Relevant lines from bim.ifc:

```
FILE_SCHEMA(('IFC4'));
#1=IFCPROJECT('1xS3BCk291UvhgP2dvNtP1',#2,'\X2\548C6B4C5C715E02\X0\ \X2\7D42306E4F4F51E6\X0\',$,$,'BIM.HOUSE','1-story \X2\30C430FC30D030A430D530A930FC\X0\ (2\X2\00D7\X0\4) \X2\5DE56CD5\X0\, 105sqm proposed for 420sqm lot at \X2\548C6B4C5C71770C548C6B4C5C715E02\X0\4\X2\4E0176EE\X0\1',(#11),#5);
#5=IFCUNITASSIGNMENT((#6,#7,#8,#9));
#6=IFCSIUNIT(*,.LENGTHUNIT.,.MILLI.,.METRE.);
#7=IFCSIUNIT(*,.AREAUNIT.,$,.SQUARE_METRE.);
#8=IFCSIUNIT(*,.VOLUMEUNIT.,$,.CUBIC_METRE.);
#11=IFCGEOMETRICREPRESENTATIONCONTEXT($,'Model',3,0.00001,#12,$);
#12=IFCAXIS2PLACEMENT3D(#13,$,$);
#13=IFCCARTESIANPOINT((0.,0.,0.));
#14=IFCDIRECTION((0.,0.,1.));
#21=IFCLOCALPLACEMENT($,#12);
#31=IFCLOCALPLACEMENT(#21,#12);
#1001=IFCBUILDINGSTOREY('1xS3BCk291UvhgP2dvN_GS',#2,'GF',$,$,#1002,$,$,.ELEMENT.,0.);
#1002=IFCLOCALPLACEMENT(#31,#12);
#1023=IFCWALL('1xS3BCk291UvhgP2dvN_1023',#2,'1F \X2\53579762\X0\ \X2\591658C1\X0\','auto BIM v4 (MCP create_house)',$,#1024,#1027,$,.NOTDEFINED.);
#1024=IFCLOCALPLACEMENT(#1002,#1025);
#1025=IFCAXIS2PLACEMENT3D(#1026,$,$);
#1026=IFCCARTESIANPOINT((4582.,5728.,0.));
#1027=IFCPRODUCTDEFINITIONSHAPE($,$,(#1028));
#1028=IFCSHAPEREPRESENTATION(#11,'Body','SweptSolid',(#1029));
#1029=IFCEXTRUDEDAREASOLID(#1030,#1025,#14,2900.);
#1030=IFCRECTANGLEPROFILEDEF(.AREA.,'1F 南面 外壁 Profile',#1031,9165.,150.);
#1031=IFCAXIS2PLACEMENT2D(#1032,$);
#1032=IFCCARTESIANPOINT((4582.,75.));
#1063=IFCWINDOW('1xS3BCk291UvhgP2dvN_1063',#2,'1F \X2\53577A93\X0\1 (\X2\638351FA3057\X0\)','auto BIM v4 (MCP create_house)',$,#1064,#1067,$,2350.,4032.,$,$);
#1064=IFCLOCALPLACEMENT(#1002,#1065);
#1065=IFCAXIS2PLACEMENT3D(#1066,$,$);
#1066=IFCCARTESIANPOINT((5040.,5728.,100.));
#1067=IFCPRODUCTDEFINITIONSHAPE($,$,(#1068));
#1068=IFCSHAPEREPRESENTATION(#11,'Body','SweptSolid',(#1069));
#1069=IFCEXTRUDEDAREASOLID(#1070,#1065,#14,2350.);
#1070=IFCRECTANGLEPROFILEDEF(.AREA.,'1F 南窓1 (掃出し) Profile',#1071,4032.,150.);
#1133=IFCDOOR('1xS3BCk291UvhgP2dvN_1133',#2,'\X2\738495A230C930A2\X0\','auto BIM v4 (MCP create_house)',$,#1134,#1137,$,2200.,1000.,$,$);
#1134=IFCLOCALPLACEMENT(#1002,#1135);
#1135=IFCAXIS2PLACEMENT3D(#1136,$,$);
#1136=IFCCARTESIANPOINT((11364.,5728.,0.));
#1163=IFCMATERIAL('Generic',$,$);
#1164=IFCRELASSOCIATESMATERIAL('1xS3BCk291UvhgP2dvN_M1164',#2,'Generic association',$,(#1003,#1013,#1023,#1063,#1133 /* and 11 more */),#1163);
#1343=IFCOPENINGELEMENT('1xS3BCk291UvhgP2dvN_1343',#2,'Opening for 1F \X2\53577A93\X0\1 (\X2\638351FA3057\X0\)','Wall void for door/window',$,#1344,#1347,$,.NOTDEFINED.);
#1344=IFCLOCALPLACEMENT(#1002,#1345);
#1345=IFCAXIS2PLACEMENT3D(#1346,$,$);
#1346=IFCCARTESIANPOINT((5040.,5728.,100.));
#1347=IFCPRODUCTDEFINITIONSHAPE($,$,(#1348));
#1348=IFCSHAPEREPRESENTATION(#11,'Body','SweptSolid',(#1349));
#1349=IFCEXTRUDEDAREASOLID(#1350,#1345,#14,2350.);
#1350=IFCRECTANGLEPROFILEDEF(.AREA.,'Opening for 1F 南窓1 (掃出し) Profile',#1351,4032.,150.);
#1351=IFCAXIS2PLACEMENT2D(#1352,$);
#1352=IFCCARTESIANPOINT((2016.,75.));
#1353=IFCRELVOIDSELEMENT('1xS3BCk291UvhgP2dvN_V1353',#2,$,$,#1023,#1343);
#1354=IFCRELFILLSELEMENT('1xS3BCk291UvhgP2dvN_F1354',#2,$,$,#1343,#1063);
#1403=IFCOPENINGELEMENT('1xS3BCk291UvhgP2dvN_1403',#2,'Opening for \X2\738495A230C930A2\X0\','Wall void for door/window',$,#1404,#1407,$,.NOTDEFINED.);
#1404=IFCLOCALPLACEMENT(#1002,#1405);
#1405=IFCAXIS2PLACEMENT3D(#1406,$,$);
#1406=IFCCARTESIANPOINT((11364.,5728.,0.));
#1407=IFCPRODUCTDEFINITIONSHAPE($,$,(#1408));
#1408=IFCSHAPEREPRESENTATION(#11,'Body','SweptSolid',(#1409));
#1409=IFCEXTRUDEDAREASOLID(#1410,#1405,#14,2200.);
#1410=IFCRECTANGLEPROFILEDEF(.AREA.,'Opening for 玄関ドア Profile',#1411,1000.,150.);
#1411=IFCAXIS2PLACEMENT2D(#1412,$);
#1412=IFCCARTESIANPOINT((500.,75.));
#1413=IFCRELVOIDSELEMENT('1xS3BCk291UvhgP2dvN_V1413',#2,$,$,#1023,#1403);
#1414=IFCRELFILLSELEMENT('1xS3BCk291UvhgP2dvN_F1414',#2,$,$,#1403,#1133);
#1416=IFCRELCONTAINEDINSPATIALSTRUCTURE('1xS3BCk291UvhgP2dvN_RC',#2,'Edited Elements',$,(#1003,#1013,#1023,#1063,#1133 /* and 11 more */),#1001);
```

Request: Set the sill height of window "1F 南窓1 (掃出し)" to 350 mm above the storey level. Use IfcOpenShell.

```python
import numpy as np
import ifcopenshell
import ifcopenshell.api.geometry
import ifcopenshell.geom
import ifcopenshell.util.element
import ifcopenshell.util.placement
import ifcopenshell.util.shape
import ifcopenshell.util.unit

model = ifcopenshell.open("bim.ifc")
unit_scale = ifcopenshell.util.unit.calculate_unit_scale(model)

window = model.by_guid("1xS3BCk291UvhgP2dvN_1063")
opening = window.FillsVoids[0].RelatingOpeningElement
storey = ifcopenshell.util.element.get_container(window, ifc_class="IfcBuildingStorey")
level = ifcopenshell.util.placement.get_local_placement(storey.ObjectPlacement)[2, 3]

# The opening's origin need not be at the sill, so measure its lowest point.
shape = ifcopenshell.geom.create_shape(ifcopenshell.geom.settings(), opening)
bottom = ifcopenshell.util.shape.get_shape_bottom_elevation(shape, shape.geometry) / unit_scale
dz = level + 0.35 / unit_scale - bottom

shift = np.array([0.0, 0.0, dz])
# The window is not placed relative to its opening, so move both.
for product in (opening, window):
    matrix = ifcopenshell.util.placement.get_local_placement(product.ObjectPlacement)
    matrix[:3, 3] += shift
    ifcopenshell.api.geometry.edit_object_placement(model, product=product, matrix=matrix, is_si=False)

print(f"moved by {dz * unit_scale:+.3f} m")

model.write("bim-out.ifc")
```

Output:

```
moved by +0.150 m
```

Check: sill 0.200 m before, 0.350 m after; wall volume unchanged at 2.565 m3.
